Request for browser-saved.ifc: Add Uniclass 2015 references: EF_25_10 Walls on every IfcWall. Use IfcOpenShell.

First a look at what the model holds.

```python
import ifcopenshell

model = ifcopenshell.open("browser-saved.ifc")
print(model.schema)
print("classifications:", [c.Name for c in model.by_type("IfcClassification")])
for ifc_class in ("IfcDoor", "IfcRoof", "IfcStair", "IfcWall", "IfcWindow"):
    print(ifc_class, len(model.by_type(ifc_class)))
```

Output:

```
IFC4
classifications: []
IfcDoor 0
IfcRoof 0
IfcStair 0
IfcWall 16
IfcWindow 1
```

```python
import ifcopenshell
import ifcopenshell.api.classification

model = ifcopenshell.open("browser-saved.ifc")

system = ifcopenshell.api.classification.add_classification(model, classification="Uniclass 2015")

codes = {
    "IfcWall": ("EF_25_10", "Walls"),
}
for ifc_class, (code, name) in codes.items():
    products = model.by_type(ifc_class)
    ifcopenshell.api.classification.add_reference(
        model, products=products, classification=system, identification=code, name=name
    )
    print(code, len(products))

model.write("browser-saved_updated.ifc")
```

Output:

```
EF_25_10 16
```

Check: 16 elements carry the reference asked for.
